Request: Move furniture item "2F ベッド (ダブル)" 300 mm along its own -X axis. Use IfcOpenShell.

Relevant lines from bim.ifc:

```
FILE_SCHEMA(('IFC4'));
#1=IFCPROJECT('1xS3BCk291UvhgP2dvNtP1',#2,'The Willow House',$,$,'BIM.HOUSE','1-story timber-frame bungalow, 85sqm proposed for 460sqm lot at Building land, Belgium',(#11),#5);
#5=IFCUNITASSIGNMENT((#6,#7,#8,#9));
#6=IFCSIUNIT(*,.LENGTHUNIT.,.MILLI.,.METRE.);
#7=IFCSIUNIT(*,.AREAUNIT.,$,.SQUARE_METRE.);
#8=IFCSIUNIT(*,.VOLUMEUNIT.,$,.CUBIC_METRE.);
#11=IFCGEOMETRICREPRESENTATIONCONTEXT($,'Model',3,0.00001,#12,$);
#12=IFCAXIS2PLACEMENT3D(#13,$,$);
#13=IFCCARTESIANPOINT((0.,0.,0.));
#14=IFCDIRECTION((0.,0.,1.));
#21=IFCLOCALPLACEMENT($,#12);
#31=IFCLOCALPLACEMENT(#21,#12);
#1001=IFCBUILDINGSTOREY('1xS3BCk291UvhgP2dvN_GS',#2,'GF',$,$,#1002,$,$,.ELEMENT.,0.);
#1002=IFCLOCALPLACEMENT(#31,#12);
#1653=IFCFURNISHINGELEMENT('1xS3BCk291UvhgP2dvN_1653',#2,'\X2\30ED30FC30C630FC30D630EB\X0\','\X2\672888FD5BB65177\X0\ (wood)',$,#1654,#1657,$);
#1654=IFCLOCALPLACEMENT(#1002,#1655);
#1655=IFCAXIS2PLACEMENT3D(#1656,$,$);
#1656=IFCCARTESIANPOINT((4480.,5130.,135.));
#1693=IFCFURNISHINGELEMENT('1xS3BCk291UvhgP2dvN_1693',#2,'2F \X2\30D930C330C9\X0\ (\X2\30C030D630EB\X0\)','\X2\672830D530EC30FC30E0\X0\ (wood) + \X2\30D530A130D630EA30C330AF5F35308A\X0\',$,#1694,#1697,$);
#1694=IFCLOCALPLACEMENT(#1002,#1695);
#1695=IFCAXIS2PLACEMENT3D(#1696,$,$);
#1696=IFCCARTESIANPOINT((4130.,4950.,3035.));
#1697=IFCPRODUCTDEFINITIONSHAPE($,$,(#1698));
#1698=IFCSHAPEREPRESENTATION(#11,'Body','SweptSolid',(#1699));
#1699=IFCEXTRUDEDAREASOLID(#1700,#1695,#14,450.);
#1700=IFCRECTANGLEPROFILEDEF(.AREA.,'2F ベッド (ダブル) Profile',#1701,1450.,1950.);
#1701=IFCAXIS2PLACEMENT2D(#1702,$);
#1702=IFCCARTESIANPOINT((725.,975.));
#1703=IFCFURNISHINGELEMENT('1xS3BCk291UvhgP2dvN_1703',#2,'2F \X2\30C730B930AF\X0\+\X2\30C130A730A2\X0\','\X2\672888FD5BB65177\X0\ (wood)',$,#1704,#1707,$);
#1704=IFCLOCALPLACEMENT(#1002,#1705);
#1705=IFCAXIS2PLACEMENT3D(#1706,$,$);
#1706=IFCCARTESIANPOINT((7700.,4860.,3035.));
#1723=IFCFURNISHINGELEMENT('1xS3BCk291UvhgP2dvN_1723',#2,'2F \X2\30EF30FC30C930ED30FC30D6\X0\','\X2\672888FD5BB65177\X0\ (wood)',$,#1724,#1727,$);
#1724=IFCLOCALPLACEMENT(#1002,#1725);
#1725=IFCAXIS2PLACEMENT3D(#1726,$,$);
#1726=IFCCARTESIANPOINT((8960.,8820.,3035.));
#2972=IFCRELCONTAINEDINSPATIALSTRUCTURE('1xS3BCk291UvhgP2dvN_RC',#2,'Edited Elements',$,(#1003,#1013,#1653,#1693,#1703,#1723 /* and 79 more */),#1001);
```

```python
import ifcopenshell
import ifcopenshell.api.geometry
import ifcopenshell.util.placement
import ifcopenshell.util.unit

model = ifcopenshell.open("bim.ifc")
unit_scale = ifcopenshell.util.unit.calculate_unit_scale(model)

item = model.by_guid("1xS3BCk291UvhgP2dvN_1693")
matrix = ifcopenshell.util.placement.get_local_placement(item.ObjectPlacement)
matrix[:3, 3] -= matrix[:3, 0] * 0.3 / unit_scale
ifcopenshell.api.geometry.edit_object_placement(model, product=item, matrix=matrix, is_si=False)

print(ifcopenshell.util.placement.get_local_placement(item.ObjectPlacement).round(3) + 0.0)

model.write("bim_rev.ifc")
```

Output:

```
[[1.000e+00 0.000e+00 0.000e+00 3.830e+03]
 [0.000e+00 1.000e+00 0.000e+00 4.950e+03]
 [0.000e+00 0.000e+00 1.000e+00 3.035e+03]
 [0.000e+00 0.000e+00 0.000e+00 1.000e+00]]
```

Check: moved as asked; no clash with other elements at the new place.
